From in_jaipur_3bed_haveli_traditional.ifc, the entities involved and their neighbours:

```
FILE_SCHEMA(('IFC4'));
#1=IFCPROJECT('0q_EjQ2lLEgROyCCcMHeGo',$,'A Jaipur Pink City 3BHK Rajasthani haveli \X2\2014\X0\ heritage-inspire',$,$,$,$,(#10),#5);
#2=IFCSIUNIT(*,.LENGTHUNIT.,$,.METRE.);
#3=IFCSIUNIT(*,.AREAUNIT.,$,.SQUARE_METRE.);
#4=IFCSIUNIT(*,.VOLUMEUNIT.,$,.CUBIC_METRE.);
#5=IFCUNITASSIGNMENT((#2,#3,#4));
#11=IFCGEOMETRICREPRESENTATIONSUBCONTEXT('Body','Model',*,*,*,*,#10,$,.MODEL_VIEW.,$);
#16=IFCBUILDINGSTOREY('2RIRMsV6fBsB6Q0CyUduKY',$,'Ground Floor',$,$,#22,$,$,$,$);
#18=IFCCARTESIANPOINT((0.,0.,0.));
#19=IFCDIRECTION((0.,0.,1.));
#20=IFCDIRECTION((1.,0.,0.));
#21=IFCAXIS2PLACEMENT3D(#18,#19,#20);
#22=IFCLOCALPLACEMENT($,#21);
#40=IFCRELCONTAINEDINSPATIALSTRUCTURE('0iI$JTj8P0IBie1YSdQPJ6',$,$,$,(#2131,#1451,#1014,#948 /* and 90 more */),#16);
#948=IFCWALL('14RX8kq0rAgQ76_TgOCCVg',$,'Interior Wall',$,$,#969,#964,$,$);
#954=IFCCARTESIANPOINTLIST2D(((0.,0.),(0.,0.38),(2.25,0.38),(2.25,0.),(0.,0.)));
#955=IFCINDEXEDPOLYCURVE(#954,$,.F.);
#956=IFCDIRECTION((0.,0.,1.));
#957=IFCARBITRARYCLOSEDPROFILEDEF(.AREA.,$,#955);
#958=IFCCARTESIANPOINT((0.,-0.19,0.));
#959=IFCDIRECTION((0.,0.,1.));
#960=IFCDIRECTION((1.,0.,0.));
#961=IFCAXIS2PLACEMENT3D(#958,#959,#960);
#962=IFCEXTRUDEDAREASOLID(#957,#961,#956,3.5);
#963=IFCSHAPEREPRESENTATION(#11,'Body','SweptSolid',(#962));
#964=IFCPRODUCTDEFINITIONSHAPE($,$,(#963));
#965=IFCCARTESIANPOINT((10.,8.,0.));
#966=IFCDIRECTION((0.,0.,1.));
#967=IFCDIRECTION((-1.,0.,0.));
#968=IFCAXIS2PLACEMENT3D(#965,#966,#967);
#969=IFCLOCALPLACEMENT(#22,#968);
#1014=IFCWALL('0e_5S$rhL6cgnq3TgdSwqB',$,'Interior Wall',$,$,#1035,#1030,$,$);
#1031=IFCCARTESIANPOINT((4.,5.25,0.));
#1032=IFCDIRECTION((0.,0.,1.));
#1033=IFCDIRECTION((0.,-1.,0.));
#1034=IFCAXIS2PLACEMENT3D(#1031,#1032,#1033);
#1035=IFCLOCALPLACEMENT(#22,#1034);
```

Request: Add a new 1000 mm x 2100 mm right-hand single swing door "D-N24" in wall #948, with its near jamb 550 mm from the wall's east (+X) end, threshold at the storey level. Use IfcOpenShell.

```python
import numpy as np
import ifcopenshell
import ifcopenshell.api.feature
import ifcopenshell.api.geometry
import ifcopenshell.api.root
import ifcopenshell.api.spatial
import ifcopenshell.geom
import ifcopenshell.util.element
import ifcopenshell.util.placement
import ifcopenshell.util.representation
import ifcopenshell.util.shape
import ifcopenshell.util.unit

model = ifcopenshell.open("in_jaipur_3bed_haveli_traditional.ifc")
unit_scale = ifcopenshell.util.unit.calculate_unit_scale(model)
settings = ifcopenshell.geom.settings()


def volume(element):
    """Net volume in cubic metres, openings subtracted."""
    shape = ifcopenshell.geom.create_shape(settings, element)
    return ifcopenshell.util.shape.get_volume(shape.geometry)


wall = model.by_guid("14RX8kq0rAgQ76_TgOCCVg")
storey = ifcopenshell.util.element.get_container(wall, ifc_class="IfcBuildingStorey")
context = ifcopenshell.util.representation.get_context(model, "Model", "Body", "MODEL_VIEW")
before = volume(wall)

width, height, from_end, sill = 1, 2.1, 0.55, 0.0  # metres

# The wall runs along its own X axis, and the end named is its -X end.
wall_shape = ifcopenshell.geom.create_shape(settings, wall)
x, y, z = ifcopenshell.util.shape.get_vertices(wall_shape.geometry).T
start = x.min() + from_end
face, thickness = float(y.min()), float(y.max() - y.min())
wall_matrix = ifcopenshell.util.placement.get_local_placement(wall.ObjectPlacement)
level = ifcopenshell.util.placement.get_local_placement(storey.ObjectPlacement)[2, 3]


def in_wall(x, y):
    """Placement at x, y metres in the wall's axes, at sill height."""
    matrix = wall_matrix.copy()
    matrix[:, 3] = wall_matrix @ np.array([x / unit_scale, y / unit_scale, 0.0, 1.0])
    matrix[2, 3] = level + sill / unit_scale
    return matrix


# Opening: a box that overshoots both wall faces by 50 mm.
opening = ifcopenshell.api.root.create_entity(model, ifc_class="IfcOpeningElement", predefined_type="OPENING")
box = ifcopenshell.api.geometry.add_wall_representation(
    model, context=context, length=width, height=height, thickness=thickness + 0.1
)
ifcopenshell.api.geometry.assign_representation(model, product=opening, representation=box)
ifcopenshell.api.geometry.edit_object_placement(model, product=opening, matrix=in_wall(start, face - 0.05), is_si=False)
ifcopenshell.api.feature.add_feature(model, feature=opening, element=wall)

door = ifcopenshell.api.root.create_entity(model, ifc_class="IfcDoor", name="D-N24", predefined_type="DOOR")
door.OverallWidth, door.OverallHeight = width / unit_scale, height / unit_scale
door.OperationType = "SINGLE_SWING_RIGHT"
body = ifcopenshell.api.geometry.add_door_representation(
    model,
    context=context,
    overall_width=door.OverallWidth,
    overall_height=door.OverallHeight,
    operation_type="SINGLE_SWING_RIGHT",
    lining_properties={"LiningDepth": thickness / unit_scale, "ThresholdDepth": thickness / unit_scale},
)
ifcopenshell.api.geometry.assign_representation(model, product=door, representation=body)
ifcopenshell.api.spatial.assign_container(model, products=[door], relating_structure=storey)
ifcopenshell.api.feature.add_filling(model, opening=opening, element=door)

# The lining spans the wall, so the door starts at the wall face.
ifcopenshell.api.geometry.edit_object_placement(model, product=door, matrix=in_wall(start, face), is_si=False)

after = volume(wall)

print(f"wall volume {before:.3f} -> {after:.3f} m3")

model.write("in_jaipur_3bed_haveli_traditional_edited.ifc")
```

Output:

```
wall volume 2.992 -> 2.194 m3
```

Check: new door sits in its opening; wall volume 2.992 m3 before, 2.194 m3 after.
